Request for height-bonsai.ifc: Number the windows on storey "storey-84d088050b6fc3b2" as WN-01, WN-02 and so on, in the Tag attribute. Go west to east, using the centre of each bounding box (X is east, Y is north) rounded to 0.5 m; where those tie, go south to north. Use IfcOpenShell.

First a look at what the model holds.

```python
import ifcopenshell
import ifcopenshell.util.element
import ifcopenshell.util.placement

model = ifcopenshell.open("height-bonsai.ifc")
print(model.schema)
storey = next(s for s in model.by_type("IfcBuildingStorey") if s.Name == "storey-84d088050b6fc3b2")
windows = [e for e in ifcopenshell.util.element.get_decomposition(storey) if e.is_a("IfcWindow")]
for e in sorted(windows, key=lambda e: e.id()):
    origin = ifcopenshell.util.placement.get_local_placement(e.ObjectPlacement)[:3, 3]
    print(e.id(), e.Tag, e.Name, origin.round(2) + 0.0, sep=" | ")
```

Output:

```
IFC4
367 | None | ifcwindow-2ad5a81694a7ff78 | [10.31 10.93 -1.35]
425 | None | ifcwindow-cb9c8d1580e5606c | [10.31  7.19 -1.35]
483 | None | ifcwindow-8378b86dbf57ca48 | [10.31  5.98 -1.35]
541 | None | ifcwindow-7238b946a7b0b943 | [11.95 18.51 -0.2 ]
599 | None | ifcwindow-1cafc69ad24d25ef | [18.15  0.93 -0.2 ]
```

```python
import ifcopenshell
import ifcopenshell.geom
import ifcopenshell.util.element
import ifcopenshell.util.shape

model = ifcopenshell.open("height-bonsai.ifc")
settings = ifcopenshell.geom.settings()
settings.set("use-world-coords", True)


def centre(element):
    shape = ifcopenshell.geom.create_shape(settings, element)
    return ifcopenshell.util.shape.get_bbox_centroid(shape.geometry)


storey = next(s for s in model.by_type("IfcBuildingStorey") if s.Name == "storey-84d088050b6fc3b2")
windows = [e for e in ifcopenshell.util.element.get_decomposition(storey) if e.is_a("IfcWindow")]

# Insertion points can sit at a corner or the storey origin, so sort by the geometry (in metres).
centres = {e: centre(e) for e in windows}
windows.sort(key=lambda e: (round(centres[e][0] / 0.5), centres[e][1]))

for i, e in enumerate(windows, start=1):
    number = f"WN-{i:02d}"
    e.Tag = number
    print(e.id(), number)

model.write("height-bonsai_v2.ifc")
```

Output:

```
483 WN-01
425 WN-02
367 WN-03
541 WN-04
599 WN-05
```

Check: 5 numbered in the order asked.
